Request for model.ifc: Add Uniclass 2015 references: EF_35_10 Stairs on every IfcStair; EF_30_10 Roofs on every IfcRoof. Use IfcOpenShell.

First a look at what the model holds.

```python
import ifcopenshell

model = ifcopenshell.open("model.ifc")
print(model.schema)
print("classifications:", [c.Name for c in model.by_type("IfcClassification")])
for ifc_class in ("IfcDoor", "IfcRoof", "IfcStair", "IfcWall", "IfcWindow"):
    print(ifc_class, len(model.by_type(ifc_class)))
```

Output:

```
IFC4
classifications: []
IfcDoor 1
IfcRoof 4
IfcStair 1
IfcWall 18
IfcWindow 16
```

```python
import ifcopenshell
import ifcopenshell.api.classification

model = ifcopenshell.open("model.ifc")

system = ifcopenshell.api.classification.add_classification(model, classification="Uniclass 2015")

codes = {
    "IfcStair": ("EF_35_10", "Stairs"),
    "IfcRoof": ("EF_30_10", "Roofs"),
}
for ifc_class, (code, name) in codes.items():
    products = model.by_type(ifc_class)
    ifcopenshell.api.classification.add_reference(
        model, products=products, classification=system, identification=code, name=name
    )
    print(code, len(products))

model.write("model_v2.ifc")
```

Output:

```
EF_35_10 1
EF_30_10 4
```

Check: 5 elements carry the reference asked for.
